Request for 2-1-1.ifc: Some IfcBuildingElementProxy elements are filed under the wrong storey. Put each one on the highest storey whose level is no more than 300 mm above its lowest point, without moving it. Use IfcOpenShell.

First a look at what the model holds.

```python
import ifcopenshell
import ifcopenshell.util.element
import ifcopenshell.util.placement

model = ifcopenshell.open("2-1-1.ifc")
print(model.schema)
for storey in model.by_type("IfcBuildingStorey"):
    level = ifcopenshell.util.placement.get_storey_elevation(storey)
    count = sum(e.is_a("IfcBuildingElementProxy") for e in ifcopenshell.util.element.get_contained(storey))
    print(storey.id(), storey.Name, round(level, 3), count, sep=" | ")
```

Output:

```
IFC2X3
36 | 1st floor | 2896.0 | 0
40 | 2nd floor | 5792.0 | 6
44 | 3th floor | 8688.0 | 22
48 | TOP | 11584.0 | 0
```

```python
import ifcopenshell
import ifcopenshell.api.spatial
import ifcopenshell.geom
import ifcopenshell.util.element
import ifcopenshell.util.placement
import ifcopenshell.util.shape
import ifcopenshell.util.unit

model = ifcopenshell.open("2-1-1.ifc")
unit_scale = ifcopenshell.util.unit.calculate_unit_scale(model)
settings = ifcopenshell.geom.settings()

levels = sorted(
    ((ifcopenshell.util.placement.get_storey_elevation(s) * unit_scale, s) for s in model.by_type("IfcBuildingStorey")),
    key=lambda pair: pair[0],
)

for e in model.by_type("IfcBuildingElementProxy"):
    current = e.ContainedInStructure[0].RelatingStructure if e.ContainedInStructure else None
    if current is None or not current.is_a("IfcBuildingStorey"):
        continue
    shape = ifcopenshell.geom.create_shape(settings, e)
    bottom = ifcopenshell.util.shape.get_shape_bottom_elevation(shape, shape.geometry)
    below = [s for level, s in levels if level <= bottom + 0.3]
    storey = below[-1] if below else levels[0][1]
    if storey != current:
        # assign_container keeps the world position.
        ifcopenshell.api.spatial.assign_container(model, products=[e], relating_structure=storey)
        print(e.id(), current.Name, "->", storey.Name)

model.write("2-1-1_v2.ifc")
```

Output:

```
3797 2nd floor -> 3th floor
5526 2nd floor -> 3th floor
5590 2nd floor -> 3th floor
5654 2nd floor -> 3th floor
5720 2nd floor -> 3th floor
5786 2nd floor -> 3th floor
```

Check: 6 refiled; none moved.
